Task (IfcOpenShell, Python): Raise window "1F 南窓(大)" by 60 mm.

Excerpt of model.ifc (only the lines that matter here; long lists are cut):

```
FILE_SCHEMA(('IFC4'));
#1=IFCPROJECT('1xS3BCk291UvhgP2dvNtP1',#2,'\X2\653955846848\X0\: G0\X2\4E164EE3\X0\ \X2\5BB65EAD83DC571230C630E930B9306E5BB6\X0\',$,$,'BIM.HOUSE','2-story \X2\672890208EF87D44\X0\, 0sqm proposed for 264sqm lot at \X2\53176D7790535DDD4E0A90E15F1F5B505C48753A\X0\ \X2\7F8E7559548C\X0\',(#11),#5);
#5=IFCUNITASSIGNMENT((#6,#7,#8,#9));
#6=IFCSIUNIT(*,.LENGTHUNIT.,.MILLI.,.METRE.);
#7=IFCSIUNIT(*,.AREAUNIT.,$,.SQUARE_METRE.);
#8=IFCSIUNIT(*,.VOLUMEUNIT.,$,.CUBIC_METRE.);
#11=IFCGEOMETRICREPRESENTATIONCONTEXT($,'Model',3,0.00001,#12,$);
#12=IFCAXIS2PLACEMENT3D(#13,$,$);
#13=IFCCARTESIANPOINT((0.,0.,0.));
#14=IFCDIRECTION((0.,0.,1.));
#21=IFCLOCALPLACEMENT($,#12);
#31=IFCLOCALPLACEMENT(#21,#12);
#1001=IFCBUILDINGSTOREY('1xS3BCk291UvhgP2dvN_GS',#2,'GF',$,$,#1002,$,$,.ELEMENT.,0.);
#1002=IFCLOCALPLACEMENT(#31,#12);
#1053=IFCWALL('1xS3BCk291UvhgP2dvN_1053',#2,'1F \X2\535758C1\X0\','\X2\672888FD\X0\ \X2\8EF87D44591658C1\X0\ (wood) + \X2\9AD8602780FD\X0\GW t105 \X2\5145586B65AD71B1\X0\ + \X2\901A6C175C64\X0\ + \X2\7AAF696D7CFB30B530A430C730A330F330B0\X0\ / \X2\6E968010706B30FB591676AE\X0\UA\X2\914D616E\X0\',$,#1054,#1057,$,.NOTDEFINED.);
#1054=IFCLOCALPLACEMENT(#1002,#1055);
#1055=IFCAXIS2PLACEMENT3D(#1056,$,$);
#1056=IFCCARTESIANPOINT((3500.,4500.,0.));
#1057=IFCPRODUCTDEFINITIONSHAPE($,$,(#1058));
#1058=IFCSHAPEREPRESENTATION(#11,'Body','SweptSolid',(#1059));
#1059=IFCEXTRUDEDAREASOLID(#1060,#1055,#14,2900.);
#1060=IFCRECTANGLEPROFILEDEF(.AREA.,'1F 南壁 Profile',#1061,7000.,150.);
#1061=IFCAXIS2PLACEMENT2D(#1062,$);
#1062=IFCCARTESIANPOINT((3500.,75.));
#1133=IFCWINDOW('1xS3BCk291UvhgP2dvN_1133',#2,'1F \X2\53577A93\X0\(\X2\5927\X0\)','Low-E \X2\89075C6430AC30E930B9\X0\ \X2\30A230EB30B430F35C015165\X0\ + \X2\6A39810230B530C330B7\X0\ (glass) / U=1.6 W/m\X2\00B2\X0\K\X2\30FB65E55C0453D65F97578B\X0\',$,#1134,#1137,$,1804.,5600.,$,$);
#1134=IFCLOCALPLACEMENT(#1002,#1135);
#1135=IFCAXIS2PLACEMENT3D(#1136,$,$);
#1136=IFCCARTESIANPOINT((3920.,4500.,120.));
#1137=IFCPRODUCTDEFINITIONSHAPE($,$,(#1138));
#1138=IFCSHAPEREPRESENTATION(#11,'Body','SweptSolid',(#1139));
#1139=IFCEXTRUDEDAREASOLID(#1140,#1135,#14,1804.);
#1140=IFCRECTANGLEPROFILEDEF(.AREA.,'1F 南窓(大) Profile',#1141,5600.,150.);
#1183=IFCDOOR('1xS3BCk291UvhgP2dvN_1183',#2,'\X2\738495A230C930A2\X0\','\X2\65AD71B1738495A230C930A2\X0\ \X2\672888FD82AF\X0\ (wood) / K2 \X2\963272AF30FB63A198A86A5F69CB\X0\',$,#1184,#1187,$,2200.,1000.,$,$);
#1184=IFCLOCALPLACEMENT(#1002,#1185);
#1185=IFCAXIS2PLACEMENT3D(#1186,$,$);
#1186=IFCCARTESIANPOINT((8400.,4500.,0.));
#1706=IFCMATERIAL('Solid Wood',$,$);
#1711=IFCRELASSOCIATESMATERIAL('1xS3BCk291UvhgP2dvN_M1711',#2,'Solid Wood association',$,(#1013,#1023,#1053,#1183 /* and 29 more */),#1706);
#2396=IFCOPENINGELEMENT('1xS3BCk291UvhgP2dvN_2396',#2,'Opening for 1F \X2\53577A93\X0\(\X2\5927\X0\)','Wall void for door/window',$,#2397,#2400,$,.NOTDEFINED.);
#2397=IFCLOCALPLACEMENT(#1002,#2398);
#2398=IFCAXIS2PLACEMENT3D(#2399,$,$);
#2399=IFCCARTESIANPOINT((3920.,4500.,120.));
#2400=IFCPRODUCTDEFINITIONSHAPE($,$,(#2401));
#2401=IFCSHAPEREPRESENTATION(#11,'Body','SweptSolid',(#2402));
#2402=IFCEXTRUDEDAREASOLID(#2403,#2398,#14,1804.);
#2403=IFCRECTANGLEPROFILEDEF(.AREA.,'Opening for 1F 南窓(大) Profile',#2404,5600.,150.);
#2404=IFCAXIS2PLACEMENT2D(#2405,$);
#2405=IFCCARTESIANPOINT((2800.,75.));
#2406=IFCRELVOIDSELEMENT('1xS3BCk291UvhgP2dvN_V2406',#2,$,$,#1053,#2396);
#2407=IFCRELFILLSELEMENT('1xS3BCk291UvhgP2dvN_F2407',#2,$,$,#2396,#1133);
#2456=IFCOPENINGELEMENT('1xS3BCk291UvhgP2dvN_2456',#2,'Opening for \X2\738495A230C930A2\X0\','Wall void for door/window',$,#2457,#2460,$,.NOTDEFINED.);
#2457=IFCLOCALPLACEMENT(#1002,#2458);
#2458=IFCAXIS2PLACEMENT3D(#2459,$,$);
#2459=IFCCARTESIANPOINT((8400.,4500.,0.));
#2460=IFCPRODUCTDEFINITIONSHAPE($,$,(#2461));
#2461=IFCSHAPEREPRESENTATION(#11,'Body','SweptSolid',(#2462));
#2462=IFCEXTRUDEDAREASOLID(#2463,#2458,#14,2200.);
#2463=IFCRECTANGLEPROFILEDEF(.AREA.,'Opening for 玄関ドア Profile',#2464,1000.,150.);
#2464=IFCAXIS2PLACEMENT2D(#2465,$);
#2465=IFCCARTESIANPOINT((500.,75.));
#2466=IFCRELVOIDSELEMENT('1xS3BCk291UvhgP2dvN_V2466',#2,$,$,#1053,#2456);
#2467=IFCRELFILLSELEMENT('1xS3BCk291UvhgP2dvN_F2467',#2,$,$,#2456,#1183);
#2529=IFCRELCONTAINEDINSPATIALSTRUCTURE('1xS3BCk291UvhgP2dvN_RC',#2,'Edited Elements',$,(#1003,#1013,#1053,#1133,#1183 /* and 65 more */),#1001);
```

```python
import numpy as np
import ifcopenshell
import ifcopenshell.api.geometry
import ifcopenshell.util.placement
import ifcopenshell.util.unit

model = ifcopenshell.open("model.ifc")
unit_scale = ifcopenshell.util.unit.calculate_unit_scale(model)

window = model.by_id(1133)
opening = window.FillsVoids[0].RelatingOpeningElement
dz = 0.06 / unit_scale

shift = np.array([0.0, 0.0, dz])
# The window is not placed relative to its opening, so move both.
for product in (opening, window):
    matrix = ifcopenshell.util.placement.get_local_placement(product.ObjectPlacement)
    matrix[:3, 3] += shift
    ifcopenshell.api.geometry.edit_object_placement(model, product=product, matrix=matrix, is_si=False)

print(f"moved by {dz * unit_scale:+.3f} m")

model.write("model-out.ifc")
```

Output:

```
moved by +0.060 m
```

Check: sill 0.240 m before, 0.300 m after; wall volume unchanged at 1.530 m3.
